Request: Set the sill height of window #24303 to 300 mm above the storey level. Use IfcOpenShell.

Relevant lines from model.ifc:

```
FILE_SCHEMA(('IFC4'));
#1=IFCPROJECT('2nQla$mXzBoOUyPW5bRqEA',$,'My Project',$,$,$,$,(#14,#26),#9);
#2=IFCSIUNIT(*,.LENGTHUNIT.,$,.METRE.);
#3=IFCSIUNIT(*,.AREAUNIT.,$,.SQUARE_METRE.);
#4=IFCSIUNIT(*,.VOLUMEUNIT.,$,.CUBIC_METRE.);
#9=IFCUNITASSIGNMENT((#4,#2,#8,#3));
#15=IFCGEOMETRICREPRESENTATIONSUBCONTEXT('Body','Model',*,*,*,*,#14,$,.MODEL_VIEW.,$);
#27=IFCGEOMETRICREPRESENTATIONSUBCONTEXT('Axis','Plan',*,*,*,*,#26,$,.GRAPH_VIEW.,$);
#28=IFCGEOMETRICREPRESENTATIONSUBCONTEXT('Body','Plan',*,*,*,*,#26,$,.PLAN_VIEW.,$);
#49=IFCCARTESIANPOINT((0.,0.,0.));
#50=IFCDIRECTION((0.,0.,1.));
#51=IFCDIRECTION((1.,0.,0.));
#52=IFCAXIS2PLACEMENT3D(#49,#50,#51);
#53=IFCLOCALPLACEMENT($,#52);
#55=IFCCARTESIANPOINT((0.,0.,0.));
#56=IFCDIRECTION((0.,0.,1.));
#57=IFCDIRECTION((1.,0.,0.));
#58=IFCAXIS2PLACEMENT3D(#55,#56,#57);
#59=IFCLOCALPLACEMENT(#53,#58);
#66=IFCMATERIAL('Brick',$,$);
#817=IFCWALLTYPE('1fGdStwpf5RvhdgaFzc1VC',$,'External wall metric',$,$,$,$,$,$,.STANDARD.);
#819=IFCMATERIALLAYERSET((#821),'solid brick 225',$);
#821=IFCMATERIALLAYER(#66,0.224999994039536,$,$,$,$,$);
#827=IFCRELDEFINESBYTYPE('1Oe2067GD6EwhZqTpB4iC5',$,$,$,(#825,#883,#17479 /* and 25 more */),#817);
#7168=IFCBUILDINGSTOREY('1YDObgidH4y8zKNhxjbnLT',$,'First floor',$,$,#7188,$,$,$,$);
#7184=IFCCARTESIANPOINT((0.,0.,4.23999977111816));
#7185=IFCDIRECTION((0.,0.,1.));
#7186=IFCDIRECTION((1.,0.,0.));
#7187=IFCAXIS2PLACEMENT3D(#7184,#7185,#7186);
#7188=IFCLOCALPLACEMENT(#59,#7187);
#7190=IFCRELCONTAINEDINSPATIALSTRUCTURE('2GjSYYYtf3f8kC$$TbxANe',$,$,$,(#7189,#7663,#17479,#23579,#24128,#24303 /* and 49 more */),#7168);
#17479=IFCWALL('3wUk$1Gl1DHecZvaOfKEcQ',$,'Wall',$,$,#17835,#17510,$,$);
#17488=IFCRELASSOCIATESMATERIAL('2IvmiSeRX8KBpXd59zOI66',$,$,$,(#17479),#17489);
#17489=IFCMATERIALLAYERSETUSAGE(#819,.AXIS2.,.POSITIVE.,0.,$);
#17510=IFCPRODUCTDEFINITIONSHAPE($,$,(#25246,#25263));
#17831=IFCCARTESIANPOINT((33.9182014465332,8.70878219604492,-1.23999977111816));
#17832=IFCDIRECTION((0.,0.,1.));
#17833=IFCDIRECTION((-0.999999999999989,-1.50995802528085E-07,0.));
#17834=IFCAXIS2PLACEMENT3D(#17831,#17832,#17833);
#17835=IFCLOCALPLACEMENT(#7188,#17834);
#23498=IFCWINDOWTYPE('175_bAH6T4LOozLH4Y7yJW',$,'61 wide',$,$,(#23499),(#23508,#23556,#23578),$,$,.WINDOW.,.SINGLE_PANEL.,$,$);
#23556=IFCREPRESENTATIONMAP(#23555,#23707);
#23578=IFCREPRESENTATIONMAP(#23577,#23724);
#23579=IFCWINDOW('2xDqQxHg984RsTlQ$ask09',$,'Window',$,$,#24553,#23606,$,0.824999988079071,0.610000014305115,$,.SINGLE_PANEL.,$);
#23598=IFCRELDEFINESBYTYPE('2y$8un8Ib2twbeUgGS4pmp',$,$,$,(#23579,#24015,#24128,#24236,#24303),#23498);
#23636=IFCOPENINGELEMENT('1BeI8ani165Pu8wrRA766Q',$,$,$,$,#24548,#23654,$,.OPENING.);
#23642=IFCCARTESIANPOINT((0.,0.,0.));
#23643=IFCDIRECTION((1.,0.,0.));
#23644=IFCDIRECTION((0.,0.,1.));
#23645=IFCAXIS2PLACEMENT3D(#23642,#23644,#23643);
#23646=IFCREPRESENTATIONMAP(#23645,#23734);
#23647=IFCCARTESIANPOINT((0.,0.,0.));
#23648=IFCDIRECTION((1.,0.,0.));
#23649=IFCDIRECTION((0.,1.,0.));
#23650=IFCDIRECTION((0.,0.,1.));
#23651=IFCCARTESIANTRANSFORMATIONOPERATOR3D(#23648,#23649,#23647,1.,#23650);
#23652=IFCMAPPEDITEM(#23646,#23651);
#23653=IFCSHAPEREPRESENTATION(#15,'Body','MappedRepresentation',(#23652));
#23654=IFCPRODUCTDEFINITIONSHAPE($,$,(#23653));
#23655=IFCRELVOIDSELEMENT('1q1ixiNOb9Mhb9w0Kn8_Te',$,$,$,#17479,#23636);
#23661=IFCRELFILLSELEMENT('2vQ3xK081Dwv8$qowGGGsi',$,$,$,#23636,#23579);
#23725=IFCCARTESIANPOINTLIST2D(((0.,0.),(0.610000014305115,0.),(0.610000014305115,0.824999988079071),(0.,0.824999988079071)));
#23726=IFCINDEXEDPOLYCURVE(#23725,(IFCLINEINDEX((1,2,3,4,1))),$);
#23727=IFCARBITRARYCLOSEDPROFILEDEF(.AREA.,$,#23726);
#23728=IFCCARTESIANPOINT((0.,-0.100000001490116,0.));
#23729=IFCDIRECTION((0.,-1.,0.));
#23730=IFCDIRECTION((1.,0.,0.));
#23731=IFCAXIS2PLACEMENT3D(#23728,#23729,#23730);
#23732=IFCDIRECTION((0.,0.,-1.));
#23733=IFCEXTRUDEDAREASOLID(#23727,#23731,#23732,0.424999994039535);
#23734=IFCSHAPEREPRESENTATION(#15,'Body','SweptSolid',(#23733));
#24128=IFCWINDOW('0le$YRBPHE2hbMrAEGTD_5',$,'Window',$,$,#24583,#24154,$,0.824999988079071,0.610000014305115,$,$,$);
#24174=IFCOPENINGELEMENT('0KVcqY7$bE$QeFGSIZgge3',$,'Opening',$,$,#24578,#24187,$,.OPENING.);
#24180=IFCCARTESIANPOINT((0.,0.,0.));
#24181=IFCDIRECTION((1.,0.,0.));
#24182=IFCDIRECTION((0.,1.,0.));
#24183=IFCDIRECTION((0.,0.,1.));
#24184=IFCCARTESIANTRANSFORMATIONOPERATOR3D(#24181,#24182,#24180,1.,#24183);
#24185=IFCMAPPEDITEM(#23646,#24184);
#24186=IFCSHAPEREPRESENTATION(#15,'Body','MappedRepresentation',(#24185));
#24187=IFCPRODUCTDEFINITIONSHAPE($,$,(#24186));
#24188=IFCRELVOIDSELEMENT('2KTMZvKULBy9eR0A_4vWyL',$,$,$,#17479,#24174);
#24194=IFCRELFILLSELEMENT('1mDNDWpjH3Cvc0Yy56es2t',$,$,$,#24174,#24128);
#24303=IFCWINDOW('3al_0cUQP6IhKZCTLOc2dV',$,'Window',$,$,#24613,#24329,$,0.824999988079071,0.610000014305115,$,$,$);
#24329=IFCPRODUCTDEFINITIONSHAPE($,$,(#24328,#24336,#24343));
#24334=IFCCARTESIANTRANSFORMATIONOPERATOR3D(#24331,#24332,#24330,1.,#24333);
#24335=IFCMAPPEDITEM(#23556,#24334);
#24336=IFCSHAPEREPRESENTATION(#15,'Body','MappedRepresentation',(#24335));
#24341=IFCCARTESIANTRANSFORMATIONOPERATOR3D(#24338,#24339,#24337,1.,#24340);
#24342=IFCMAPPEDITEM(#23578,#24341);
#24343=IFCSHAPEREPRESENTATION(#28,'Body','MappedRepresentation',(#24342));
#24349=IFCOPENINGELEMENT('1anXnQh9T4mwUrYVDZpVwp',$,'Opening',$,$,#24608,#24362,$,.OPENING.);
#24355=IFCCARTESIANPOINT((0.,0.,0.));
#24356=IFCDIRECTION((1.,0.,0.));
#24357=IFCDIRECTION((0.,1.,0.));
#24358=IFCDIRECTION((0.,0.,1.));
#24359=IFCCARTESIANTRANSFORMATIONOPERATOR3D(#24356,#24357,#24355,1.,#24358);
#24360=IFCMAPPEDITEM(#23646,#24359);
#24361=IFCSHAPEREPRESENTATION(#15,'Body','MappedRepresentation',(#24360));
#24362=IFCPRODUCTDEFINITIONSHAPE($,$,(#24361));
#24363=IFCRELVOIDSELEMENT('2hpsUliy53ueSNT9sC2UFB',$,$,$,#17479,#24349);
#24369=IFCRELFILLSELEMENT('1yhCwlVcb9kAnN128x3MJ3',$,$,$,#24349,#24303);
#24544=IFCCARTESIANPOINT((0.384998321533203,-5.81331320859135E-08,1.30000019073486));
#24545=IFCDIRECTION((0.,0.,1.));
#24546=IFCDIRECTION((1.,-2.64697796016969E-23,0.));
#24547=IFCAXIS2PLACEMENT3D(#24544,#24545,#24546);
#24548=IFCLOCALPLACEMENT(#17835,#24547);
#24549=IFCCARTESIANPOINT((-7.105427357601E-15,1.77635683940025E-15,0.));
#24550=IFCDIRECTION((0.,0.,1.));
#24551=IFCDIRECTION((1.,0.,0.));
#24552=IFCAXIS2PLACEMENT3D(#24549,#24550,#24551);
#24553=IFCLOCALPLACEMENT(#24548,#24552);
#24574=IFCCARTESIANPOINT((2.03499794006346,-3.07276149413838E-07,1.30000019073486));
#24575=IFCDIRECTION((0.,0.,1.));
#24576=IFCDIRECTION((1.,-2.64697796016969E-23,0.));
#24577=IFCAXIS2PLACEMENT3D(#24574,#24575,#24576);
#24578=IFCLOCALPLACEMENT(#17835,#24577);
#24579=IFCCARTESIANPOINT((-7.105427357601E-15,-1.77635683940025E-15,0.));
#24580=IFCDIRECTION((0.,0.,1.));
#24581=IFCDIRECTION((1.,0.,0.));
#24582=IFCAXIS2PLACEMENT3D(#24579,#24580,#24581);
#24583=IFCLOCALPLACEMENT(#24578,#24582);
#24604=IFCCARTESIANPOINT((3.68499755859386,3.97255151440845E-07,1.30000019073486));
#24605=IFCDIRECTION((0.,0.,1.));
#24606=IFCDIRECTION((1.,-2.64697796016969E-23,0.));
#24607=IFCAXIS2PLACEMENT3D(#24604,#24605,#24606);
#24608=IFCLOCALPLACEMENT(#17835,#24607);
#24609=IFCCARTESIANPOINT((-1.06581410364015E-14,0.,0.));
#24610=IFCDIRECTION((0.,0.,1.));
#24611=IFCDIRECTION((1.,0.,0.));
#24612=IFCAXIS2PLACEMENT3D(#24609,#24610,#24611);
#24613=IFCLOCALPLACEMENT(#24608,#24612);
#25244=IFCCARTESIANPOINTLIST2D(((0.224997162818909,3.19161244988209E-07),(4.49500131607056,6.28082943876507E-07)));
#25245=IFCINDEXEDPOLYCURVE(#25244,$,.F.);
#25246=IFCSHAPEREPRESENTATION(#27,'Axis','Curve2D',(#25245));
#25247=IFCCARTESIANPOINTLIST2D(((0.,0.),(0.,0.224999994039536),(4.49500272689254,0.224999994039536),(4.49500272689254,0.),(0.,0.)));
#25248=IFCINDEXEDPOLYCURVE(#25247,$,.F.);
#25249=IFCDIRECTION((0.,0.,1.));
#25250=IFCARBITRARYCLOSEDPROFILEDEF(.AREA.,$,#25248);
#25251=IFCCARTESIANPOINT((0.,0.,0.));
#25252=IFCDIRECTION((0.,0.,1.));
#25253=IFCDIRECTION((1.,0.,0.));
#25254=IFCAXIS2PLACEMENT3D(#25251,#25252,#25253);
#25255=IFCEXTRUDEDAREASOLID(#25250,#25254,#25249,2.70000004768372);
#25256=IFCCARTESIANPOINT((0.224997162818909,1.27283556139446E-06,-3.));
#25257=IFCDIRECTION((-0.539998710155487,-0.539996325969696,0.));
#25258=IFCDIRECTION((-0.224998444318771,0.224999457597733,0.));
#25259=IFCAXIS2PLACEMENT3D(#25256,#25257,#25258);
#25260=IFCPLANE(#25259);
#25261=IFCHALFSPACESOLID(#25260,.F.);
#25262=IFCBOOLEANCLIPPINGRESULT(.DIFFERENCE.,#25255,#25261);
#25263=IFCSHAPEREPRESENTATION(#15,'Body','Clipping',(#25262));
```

```python
import numpy as np
import ifcopenshell
import ifcopenshell.api.geometry
import ifcopenshell.geom
import ifcopenshell.util.element
import ifcopenshell.util.placement
import ifcopenshell.util.shape
import ifcopenshell.util.unit

model = ifcopenshell.open("model.ifc")
unit_scale = ifcopenshell.util.unit.calculate_unit_scale(model)

window = model.by_guid("3al_0cUQP6IhKZCTLOc2dV")
opening = window.FillsVoids[0].RelatingOpeningElement
storey = ifcopenshell.util.element.get_container(window, ifc_class="IfcBuildingStorey")
level = ifcopenshell.util.placement.get_local_placement(storey.ObjectPlacement)[2, 3]

# The opening's origin need not be at the sill, so measure its lowest point.
shape = ifcopenshell.geom.create_shape(ifcopenshell.geom.settings(), opening)
bottom = ifcopenshell.util.shape.get_shape_bottom_elevation(shape, shape.geometry) / unit_scale
dz = level + 0.3 / unit_scale - bottom

shift = np.array([0.0, 0.0, dz])
# The window is placed relative to its opening, so it follows when the opening moves.
matrix = ifcopenshell.util.placement.get_local_placement(opening.ObjectPlacement)
matrix[:3, 3] += shift
ifcopenshell.api.geometry.edit_object_placement(
    model, product=opening, matrix=matrix, is_si=False, should_transform_children=True
)

print(f"moved by {dz * unit_scale:+.3f} m")

model.write("model_rev.ifc")
```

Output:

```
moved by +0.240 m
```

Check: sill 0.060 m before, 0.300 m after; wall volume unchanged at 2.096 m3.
